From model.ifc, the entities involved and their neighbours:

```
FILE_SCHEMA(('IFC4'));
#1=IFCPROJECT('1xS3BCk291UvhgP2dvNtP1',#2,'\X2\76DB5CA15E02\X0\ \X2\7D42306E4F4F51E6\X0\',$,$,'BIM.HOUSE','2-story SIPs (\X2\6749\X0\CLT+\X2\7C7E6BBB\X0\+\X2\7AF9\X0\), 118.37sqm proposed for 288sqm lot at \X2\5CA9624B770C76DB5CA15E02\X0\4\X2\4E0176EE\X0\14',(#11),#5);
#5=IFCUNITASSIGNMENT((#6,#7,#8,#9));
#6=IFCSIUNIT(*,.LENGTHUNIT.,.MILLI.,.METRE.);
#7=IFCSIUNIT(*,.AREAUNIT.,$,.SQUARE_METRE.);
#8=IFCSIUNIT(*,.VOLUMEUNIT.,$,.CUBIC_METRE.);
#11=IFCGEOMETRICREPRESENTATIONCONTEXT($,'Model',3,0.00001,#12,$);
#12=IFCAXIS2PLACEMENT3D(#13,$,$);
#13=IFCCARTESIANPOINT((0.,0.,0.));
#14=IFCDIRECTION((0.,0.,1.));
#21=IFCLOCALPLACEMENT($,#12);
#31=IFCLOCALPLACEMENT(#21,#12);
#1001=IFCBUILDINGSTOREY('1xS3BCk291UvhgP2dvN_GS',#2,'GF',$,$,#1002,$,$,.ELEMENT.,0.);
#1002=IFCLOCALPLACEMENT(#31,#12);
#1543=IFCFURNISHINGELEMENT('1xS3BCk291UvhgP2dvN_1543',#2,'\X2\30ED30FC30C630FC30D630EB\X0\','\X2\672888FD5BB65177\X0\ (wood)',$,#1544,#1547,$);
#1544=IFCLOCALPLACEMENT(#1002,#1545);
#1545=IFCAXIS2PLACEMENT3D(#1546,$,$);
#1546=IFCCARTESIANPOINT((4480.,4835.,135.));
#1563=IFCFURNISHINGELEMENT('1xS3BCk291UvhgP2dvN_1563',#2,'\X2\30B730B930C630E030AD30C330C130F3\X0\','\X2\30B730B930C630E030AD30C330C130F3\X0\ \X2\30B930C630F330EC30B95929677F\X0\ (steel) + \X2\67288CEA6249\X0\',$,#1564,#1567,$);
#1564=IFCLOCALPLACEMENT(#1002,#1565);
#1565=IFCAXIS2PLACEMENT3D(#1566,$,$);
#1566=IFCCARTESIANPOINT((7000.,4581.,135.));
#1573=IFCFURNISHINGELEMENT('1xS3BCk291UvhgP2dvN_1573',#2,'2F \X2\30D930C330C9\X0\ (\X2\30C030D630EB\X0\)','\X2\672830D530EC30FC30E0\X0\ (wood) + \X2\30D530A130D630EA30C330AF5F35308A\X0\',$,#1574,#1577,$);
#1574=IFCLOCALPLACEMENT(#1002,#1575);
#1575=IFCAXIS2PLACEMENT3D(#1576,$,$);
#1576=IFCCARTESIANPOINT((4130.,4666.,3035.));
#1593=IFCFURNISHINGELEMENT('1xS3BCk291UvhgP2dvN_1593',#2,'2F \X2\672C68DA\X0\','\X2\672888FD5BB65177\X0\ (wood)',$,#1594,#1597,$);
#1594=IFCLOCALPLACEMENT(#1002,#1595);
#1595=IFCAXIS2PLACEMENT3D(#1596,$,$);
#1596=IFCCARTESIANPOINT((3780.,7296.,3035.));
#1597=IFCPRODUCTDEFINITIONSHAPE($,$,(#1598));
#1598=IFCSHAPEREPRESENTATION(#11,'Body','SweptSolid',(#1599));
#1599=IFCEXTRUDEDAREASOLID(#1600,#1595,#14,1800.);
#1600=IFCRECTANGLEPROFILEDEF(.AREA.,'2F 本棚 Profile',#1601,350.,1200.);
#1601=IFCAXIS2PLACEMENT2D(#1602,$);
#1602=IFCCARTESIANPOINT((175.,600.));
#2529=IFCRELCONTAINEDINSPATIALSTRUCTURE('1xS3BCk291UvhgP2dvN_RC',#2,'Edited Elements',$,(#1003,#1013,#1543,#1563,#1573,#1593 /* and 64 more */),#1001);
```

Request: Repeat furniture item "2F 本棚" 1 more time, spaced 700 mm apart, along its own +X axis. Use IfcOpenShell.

```python
import ifcopenshell
import ifcopenshell.api.geometry
import ifcopenshell.api.root
import ifcopenshell.util.element
import ifcopenshell.util.placement

model = ifcopenshell.open("model.ifc")


def reuse_history(source, copy):
    """copy_class also copies each property set's owner history, people and application; keep the originals."""
    for rel in copy.IsDefinedBy:
        if rel.is_a("IfcRelDefinesByProperties") and (history := rel.RelatingPropertyDefinition.OwnerHistory):
            rel.RelatingPropertyDefinition.OwnerHistory = source.OwnerHistory
            ifcopenshell.util.element.remove_deep2(model, history)


source = model.by_guid("1xS3BCk291UvhgP2dvN_1593")
base = ifcopenshell.util.placement.get_local_placement(source.ObjectPlacement)
step = base[:3, 0] * 700.0

for i in range(1, 2):
    copy = ifcopenshell.api.root.copy_class(model, product=source)
    copy.Representation = ifcopenshell.util.element.copy_deep(
        model, source.Representation, exclude=["IfcGeometricRepresentationContext", "IfcRepresentationMap"]
    )
    reuse_history(source, copy)
    matrix = base.copy()
    matrix[:3, 3] += i * step
    print("added at", matrix[:3, 3].round(3) + 0.0)
    ifcopenshell.api.geometry.edit_object_placement(model, product=copy, matrix=matrix, is_si=False)

model.write("model_updated.ifc")
```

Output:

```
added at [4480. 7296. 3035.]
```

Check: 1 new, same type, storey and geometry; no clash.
